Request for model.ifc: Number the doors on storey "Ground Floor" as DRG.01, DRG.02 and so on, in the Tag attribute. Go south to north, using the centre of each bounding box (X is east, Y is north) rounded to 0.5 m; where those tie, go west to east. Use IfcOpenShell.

First a look at what the model holds.

```python
import ifcopenshell
import ifcopenshell.util.element
import ifcopenshell.util.placement

model = ifcopenshell.open("model.ifc")
print(model.schema)
storey = next(s for s in model.by_type("IfcBuildingStorey") if s.Name == "Ground Floor")
doors = [e for e in ifcopenshell.util.element.get_decomposition(storey) if e.is_a("IfcDoor")]
for e in sorted(doors, key=lambda e: e.id()):
    origin = ifcopenshell.util.placement.get_local_placement(e.ObjectPlacement)[:3, 3]
    print(e.id(), e.Tag, e.Name, origin.round(2) + 0.0, sep=" | ")
```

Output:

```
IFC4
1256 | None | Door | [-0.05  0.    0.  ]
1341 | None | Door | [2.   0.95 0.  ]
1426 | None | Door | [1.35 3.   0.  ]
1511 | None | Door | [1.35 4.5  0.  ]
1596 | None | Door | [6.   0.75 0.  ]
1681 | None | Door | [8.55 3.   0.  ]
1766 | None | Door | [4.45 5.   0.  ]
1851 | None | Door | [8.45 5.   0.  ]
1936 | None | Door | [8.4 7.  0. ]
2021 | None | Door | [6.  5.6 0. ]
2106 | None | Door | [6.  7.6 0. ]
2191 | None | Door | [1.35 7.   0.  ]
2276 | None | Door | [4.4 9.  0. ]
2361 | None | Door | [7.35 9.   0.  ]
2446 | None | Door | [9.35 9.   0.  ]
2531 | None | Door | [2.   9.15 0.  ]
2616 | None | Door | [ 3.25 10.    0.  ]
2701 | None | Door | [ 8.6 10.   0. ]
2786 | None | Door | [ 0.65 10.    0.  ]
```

```python
import ifcopenshell
import ifcopenshell.geom
import ifcopenshell.util.element
import ifcopenshell.util.shape

model = ifcopenshell.open("model.ifc")
settings = ifcopenshell.geom.settings()
settings.set("use-world-coords", True)


def centre(element):
    shape = ifcopenshell.geom.create_shape(settings, element)
    return ifcopenshell.util.shape.get_bbox_centroid(shape.geometry)


storey = next(s for s in model.by_type("IfcBuildingStorey") if s.Name == "Ground Floor")
doors = [e for e in ifcopenshell.util.element.get_decomposition(storey) if e.is_a("IfcDoor")]

# Insertion points can sit at a corner or the storey origin, so sort by the geometry (in metres).
centres = {e: centre(e) for e in doors}
doors.sort(key=lambda e: (round(centres[e][1] / 0.5), centres[e][0]))

for i, e in enumerate(doors, start=1):
    number = f"DRG.{i:02d}"
    e.Tag = number
    print(e.id(), number)

model.write("model_rev.ifc")
```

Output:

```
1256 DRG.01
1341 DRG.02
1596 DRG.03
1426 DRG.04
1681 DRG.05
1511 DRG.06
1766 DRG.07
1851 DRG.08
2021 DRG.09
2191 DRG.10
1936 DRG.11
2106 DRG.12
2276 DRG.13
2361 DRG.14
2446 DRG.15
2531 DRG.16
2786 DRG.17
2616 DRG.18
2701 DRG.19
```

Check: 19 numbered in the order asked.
